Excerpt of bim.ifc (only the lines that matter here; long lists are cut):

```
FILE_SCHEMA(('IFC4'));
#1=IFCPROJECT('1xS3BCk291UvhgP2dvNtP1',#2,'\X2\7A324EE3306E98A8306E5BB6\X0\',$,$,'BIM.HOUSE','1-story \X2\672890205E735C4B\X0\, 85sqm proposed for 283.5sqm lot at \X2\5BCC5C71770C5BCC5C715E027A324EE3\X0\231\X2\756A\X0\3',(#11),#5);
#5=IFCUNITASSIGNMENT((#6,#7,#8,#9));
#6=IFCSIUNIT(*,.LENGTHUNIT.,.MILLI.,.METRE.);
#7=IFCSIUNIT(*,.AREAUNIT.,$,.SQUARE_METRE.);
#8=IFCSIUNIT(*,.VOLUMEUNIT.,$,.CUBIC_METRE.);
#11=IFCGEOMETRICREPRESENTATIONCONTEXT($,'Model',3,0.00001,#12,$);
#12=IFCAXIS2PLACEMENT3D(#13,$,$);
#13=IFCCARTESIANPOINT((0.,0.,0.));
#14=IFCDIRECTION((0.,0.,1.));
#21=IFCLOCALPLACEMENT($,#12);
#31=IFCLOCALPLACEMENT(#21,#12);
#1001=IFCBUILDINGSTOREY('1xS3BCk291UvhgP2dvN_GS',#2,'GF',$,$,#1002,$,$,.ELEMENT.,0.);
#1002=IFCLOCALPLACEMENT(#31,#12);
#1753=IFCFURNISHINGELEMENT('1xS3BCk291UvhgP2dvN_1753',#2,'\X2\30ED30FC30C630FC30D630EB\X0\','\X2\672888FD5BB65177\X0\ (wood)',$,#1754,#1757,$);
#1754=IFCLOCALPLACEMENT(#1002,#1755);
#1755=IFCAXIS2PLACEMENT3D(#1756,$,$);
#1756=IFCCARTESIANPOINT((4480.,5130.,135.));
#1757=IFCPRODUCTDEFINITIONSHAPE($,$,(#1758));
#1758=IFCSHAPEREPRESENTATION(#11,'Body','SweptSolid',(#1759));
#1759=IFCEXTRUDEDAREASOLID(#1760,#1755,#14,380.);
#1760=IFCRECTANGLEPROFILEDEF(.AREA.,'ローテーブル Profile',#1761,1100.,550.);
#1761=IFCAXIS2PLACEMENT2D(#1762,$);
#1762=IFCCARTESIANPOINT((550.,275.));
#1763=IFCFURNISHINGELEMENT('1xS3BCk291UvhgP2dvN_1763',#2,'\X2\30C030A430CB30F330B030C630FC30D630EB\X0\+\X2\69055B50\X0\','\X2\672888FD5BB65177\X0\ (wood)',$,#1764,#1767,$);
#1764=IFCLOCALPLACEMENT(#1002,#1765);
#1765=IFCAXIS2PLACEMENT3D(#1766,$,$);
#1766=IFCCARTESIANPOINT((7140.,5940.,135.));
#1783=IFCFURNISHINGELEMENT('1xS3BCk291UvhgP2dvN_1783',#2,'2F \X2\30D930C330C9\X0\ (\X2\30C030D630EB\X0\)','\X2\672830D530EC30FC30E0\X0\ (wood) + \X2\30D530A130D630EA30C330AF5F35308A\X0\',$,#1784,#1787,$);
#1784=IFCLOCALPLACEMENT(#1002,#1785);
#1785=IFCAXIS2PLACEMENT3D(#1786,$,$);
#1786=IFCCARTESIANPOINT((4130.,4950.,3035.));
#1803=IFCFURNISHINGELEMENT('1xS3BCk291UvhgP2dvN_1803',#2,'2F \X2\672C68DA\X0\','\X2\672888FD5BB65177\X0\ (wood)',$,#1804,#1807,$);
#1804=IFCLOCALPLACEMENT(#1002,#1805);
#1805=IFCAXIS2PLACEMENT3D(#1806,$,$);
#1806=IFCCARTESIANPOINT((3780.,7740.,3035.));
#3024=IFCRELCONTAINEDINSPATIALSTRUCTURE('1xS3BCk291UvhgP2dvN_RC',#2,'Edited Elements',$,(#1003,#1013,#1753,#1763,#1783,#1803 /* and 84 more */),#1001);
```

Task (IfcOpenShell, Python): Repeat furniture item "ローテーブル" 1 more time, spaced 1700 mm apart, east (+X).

```python
import numpy as np
import ifcopenshell
import ifcopenshell.api.geometry
import ifcopenshell.api.root
import ifcopenshell.util.element
import ifcopenshell.util.placement

model = ifcopenshell.open("bim.ifc")


def reuse_history(source, copy):
    """copy_class also copies each property set's owner history, people and application; keep the originals."""
    for rel in copy.IsDefinedBy:
        if rel.is_a("IfcRelDefinesByProperties") and (history := rel.RelatingPropertyDefinition.OwnerHistory):
            rel.RelatingPropertyDefinition.OwnerHistory = source.OwnerHistory
            ifcopenshell.util.element.remove_deep2(model, history)


source = model.by_id(1753)
base = ifcopenshell.util.placement.get_local_placement(source.ObjectPlacement)
step = np.array([1.0, 0.0, 0.0]) * 1700.0

for i in range(1, 2):
    copy = ifcopenshell.api.root.copy_class(model, product=source)
    copy.Representation = ifcopenshell.util.element.copy_deep(
        model, source.Representation, exclude=["IfcGeometricRepresentationContext", "IfcRepresentationMap"]
    )
    reuse_history(source, copy)
    matrix = base.copy()
    matrix[:3, 3] += i * step
    print("added at", matrix[:3, 3].round(3) + 0.0)
    ifcopenshell.api.geometry.edit_object_placement(model, product=copy, matrix=matrix, is_si=False)

model.write("bim_updated.ifc")
```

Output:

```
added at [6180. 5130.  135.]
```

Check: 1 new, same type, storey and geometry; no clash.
